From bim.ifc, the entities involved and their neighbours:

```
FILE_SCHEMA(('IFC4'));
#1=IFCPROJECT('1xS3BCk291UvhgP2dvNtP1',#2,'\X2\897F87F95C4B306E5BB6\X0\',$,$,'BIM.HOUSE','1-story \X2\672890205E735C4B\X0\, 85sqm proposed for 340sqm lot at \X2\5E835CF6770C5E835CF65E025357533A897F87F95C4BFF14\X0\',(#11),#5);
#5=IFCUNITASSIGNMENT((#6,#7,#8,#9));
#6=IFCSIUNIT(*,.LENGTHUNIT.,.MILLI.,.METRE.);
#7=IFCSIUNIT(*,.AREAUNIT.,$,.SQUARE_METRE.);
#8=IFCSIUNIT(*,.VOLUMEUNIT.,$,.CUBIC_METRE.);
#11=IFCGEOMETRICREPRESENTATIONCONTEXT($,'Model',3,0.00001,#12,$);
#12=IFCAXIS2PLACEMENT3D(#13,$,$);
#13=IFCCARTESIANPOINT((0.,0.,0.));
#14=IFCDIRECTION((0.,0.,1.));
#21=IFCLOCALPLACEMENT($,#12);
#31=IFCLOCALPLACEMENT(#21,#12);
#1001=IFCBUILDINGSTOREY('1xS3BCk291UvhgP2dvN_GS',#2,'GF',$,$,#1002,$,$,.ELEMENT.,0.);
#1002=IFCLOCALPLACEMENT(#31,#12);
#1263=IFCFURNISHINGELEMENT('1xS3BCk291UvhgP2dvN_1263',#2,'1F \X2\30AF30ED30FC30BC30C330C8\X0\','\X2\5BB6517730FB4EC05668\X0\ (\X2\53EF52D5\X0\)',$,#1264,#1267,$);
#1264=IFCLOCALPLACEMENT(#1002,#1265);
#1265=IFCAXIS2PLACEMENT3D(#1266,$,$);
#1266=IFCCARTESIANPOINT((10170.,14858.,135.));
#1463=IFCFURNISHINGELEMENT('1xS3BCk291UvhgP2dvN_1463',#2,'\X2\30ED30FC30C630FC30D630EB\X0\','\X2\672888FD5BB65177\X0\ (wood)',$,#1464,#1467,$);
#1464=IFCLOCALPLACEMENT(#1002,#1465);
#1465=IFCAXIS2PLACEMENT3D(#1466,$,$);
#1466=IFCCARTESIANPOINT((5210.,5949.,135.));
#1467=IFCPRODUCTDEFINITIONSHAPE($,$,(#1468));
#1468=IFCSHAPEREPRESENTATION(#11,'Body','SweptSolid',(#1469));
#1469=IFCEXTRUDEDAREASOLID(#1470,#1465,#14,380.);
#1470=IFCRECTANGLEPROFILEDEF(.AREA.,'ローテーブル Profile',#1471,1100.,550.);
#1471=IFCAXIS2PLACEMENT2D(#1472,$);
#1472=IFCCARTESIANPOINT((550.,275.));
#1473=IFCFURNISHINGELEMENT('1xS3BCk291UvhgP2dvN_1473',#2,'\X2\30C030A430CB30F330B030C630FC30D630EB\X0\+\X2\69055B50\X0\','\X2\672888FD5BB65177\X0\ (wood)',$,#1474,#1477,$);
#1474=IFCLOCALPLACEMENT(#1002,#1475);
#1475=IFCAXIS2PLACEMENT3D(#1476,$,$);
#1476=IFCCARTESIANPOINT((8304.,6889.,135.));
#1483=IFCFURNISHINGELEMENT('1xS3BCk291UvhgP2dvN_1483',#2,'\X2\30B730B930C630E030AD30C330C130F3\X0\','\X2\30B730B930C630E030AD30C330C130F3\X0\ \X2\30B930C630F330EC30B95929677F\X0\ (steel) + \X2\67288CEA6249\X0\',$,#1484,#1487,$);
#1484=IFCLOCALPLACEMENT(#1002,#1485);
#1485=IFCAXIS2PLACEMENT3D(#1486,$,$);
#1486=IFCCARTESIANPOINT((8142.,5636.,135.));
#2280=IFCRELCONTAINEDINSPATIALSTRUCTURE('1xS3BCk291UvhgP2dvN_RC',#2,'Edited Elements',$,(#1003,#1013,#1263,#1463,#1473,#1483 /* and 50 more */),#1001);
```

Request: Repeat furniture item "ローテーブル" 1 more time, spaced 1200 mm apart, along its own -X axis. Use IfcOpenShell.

```python
import ifcopenshell
import ifcopenshell.api.geometry
import ifcopenshell.api.root
import ifcopenshell.util.element
import ifcopenshell.util.placement
import ifcopenshell.util.unit

model = ifcopenshell.open("bim.ifc")
unit_scale = ifcopenshell.util.unit.calculate_unit_scale(model)


def reuse_history(source, copy):
    """copy_class also copies each property set's owner history, people and application; keep the originals."""
    for rel in copy.IsDefinedBy:
        if rel.is_a("IfcRelDefinesByProperties") and (history := rel.RelatingPropertyDefinition.OwnerHistory):
            rel.RelatingPropertyDefinition.OwnerHistory = source.OwnerHistory
            ifcopenshell.util.element.remove_deep2(model, history)


source = model.by_guid("1xS3BCk291UvhgP2dvN_1463")
base = ifcopenshell.util.placement.get_local_placement(source.ObjectPlacement)
step = -base[:3, 0] * 1.2 / unit_scale

for i in range(1, 2):
    copy = ifcopenshell.api.root.copy_class(model, product=source)
    copy.Representation = ifcopenshell.util.element.copy_deep(
        model, source.Representation, exclude=["IfcGeometricRepresentationContext", "IfcRepresentationMap"]
    )
    reuse_history(source, copy)
    matrix = base.copy()
    matrix[:3, 3] += i * step
    print("added at", matrix[:3, 3].round(3) + 0.0)
    ifcopenshell.api.geometry.edit_object_placement(model, product=copy, matrix=matrix, is_si=False)

model.write("bim_edited.ifc")
```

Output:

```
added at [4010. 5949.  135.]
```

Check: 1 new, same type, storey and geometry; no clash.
